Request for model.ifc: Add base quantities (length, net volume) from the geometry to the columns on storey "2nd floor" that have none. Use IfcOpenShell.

First a look at what the model holds.

```python
import ifcopenshell
import ifcopenshell.util.element
import ifcopenshell.util.unit

model = ifcopenshell.open("model.ifc")
print(model.schema)
for unit_type in ("LENGTHUNIT", "AREAUNIT", "VOLUMEUNIT"):
    print(unit_type, ifcopenshell.util.unit.calculate_unit_scale(model, unit_type))
storey = next(s for s in model.by_type("IfcBuildingStorey") if s.Name == "2nd floor")
columns = [e for e in ifcopenshell.util.element.get_decomposition(storey) if e.is_a("IfcColumn")]
for e in sorted(columns, key=lambda e: e.id()):
    print(e.id(), e.is_a(), e.Name, list(ifcopenshell.util.element.get_psets(e, qtos_only=True)), sep=" | ")
```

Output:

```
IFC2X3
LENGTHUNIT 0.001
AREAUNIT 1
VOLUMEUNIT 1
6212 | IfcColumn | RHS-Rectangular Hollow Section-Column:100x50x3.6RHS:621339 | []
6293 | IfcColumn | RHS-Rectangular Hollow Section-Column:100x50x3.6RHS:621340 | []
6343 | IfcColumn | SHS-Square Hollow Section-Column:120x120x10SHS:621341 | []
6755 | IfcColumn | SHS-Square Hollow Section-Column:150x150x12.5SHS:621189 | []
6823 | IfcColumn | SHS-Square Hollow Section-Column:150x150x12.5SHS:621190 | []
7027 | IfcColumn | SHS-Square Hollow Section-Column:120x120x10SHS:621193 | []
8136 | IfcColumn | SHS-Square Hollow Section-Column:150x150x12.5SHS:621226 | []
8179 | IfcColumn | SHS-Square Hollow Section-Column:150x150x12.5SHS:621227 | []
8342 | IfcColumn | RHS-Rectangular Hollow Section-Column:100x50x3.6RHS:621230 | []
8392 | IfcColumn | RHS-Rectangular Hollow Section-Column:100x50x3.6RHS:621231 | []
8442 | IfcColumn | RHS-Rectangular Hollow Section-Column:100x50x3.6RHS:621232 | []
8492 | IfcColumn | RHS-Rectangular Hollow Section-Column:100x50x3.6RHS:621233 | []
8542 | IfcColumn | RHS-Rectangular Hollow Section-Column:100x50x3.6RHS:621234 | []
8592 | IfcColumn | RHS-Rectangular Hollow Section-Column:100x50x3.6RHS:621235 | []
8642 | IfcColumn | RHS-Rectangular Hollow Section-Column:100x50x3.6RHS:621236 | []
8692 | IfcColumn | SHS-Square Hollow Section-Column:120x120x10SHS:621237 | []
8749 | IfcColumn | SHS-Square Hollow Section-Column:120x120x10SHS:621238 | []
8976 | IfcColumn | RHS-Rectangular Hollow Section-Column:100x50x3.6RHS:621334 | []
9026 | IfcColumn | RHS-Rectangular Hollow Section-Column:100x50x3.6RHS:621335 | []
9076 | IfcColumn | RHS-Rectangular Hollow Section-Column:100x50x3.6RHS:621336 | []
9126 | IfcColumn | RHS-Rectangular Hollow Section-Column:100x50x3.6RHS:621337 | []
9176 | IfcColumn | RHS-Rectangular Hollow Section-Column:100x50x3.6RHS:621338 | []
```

```python
import ifcopenshell
import ifcopenshell.api.pset
import ifcopenshell.geom
import ifcopenshell.util.element
import ifcopenshell.util.shape
import ifcopenshell.util.unit

model = ifcopenshell.open("model.ifc")
unit_scale = ifcopenshell.util.unit.calculate_unit_scale(model)
volume_scale = ifcopenshell.util.unit.calculate_unit_scale(model, "VOLUMEUNIT")
settings = ifcopenshell.geom.settings()

storey = next(s for s in model.by_type("IfcBuildingStorey") if s.Name == "2nd floor")
columns = [e for e in ifcopenshell.util.element.get_decomposition(storey) if e.is_a("IfcColumn")]

for e in sorted(columns, key=lambda e: e.id()):
    if ifcopenshell.util.element.get_psets(e, qtos_only=True, should_inherit=False):
        continue
    # Geometry comes back in metres, in the element's own axes.
    shape = ifcopenshell.geom.create_shape(settings, e)
    values = {
        "Length": ifcopenshell.util.shape.get_z(shape.geometry) / unit_scale,
        "NetVolume": ifcopenshell.util.shape.get_volume(shape.geometry) / volume_scale,
    }
    qto = ifcopenshell.api.pset.add_qto(model, product=e, name="BaseQuantities")
    ifcopenshell.api.pset.edit_qto(model, qto=qto, properties=values)
    print(e.id(), {k: round(v, 3) for k, v in values.items()})

model.write("model_v2.ifc")
```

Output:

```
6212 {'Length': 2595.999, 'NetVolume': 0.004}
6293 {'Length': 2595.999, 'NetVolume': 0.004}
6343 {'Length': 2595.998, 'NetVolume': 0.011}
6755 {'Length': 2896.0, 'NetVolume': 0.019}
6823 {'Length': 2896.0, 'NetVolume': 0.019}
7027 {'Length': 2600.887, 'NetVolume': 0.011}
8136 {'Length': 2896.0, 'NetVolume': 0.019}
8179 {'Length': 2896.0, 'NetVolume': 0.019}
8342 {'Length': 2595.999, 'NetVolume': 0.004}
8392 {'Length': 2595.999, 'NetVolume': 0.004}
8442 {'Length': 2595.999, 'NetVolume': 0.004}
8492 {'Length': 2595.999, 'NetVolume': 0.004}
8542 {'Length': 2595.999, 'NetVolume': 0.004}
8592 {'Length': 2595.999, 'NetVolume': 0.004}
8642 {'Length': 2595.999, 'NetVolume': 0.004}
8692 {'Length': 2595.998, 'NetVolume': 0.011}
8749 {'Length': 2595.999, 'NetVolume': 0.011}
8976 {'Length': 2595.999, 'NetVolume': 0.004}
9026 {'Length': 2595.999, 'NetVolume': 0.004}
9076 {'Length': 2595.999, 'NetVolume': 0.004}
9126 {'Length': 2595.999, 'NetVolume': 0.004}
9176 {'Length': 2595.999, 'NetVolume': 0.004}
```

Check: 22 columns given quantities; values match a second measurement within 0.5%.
